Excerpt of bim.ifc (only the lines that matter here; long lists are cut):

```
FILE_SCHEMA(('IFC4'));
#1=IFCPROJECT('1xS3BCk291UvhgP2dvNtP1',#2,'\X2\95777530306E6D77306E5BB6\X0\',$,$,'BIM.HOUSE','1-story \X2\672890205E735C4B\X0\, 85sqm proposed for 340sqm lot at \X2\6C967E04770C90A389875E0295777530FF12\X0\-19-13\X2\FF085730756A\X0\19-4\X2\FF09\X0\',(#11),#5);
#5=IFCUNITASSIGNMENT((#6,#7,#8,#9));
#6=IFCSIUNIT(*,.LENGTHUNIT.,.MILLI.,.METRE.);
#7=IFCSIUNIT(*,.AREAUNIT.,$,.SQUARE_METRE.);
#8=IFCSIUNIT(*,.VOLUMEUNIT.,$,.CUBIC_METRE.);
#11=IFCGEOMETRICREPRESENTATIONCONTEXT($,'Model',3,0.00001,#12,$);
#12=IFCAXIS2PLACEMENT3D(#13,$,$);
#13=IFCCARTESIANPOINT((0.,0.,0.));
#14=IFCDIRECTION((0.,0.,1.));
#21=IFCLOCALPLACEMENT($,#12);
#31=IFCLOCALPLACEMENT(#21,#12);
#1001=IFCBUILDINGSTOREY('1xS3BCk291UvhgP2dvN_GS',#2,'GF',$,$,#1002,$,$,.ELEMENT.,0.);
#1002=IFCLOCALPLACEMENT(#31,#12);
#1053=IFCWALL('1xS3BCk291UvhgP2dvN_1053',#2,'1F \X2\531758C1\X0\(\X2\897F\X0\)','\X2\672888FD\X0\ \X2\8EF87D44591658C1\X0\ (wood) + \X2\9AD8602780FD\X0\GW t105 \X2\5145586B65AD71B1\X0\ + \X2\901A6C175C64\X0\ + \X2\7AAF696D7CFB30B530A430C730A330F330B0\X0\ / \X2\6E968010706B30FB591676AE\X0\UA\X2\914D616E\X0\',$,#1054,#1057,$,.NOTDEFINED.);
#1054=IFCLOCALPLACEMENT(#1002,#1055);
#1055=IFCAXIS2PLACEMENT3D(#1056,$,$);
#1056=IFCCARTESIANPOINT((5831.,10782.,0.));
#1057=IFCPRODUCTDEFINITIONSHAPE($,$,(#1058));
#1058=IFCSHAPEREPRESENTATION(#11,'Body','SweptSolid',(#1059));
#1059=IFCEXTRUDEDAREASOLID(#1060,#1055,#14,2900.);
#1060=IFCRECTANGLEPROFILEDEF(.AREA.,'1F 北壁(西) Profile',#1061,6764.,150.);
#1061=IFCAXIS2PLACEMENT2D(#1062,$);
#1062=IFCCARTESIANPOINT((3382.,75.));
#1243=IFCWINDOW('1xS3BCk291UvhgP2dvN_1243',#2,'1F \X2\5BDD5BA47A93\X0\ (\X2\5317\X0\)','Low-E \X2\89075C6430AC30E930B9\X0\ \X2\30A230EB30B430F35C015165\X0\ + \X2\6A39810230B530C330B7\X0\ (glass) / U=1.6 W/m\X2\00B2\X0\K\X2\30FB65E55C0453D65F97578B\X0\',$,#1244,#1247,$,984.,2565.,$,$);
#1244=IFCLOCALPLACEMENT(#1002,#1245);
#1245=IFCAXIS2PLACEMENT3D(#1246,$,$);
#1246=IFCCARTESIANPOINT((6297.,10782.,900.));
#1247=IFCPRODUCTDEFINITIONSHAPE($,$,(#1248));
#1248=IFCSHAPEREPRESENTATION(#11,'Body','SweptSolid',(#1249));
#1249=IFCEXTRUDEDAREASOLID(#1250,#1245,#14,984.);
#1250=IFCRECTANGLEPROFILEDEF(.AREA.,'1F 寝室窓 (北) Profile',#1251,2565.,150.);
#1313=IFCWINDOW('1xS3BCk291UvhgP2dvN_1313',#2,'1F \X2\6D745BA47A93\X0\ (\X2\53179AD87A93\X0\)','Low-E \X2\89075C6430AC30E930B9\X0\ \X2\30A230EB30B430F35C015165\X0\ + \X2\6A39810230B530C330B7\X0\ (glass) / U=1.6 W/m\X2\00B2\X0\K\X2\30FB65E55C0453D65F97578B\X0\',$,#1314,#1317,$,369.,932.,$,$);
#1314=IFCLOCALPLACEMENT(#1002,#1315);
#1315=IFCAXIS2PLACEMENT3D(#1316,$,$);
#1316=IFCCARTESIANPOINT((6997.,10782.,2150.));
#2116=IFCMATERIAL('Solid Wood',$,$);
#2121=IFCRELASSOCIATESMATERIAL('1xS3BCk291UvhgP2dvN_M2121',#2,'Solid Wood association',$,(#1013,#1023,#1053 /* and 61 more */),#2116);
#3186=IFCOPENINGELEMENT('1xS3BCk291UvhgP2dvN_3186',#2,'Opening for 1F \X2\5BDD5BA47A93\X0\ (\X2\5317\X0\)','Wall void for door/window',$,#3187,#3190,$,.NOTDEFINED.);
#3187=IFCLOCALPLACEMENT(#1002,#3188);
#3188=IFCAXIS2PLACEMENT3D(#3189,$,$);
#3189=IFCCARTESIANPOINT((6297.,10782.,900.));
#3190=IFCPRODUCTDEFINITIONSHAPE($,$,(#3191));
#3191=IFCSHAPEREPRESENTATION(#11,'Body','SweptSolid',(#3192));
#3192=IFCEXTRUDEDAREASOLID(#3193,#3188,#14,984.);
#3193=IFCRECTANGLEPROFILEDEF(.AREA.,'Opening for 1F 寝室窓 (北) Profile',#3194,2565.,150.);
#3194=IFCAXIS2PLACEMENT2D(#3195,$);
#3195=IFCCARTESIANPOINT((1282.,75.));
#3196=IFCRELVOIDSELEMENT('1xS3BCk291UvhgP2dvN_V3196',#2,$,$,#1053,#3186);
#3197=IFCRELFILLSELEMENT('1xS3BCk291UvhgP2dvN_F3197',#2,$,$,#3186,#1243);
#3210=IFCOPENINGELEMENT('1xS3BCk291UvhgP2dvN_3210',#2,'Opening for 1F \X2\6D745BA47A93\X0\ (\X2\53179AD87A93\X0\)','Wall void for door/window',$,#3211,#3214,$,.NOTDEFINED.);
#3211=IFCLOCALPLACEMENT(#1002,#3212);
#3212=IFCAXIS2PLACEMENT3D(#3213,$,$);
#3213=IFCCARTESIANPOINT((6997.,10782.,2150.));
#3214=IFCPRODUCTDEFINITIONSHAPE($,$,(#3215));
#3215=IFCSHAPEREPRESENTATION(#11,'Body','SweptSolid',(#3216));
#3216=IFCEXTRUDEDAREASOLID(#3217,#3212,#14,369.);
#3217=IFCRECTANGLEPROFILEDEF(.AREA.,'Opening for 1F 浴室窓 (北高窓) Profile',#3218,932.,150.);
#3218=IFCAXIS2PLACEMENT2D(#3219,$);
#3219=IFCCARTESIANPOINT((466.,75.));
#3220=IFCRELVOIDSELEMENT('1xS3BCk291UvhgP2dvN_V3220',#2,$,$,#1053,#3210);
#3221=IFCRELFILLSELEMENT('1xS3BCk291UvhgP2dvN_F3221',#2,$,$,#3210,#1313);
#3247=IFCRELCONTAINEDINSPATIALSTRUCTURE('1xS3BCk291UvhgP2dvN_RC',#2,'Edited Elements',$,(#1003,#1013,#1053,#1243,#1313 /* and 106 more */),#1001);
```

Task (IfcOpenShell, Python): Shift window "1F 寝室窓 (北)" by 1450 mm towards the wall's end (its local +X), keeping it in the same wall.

```python
import ifcopenshell
import ifcopenshell.api.geometry
import ifcopenshell.util.placement
import ifcopenshell.util.unit

model = ifcopenshell.open("bim.ifc")
unit_scale = ifcopenshell.util.unit.calculate_unit_scale(model)

window = model.by_guid("1xS3BCk291UvhgP2dvN_1243")
opening = window.FillsVoids[0].RelatingOpeningElement
wall = opening.VoidsElements[0].RelatingBuildingElement

wall_matrix = ifcopenshell.util.placement.get_local_placement(wall.ObjectPlacement)
shift = wall_matrix[:3, 0] * 1.45 / unit_scale
before = ifcopenshell.util.placement.get_local_placement(window.ObjectPlacement)[:3, 3].copy()

# The window is not placed relative to its opening, so move both.
for product in (opening, window):
    matrix = ifcopenshell.util.placement.get_local_placement(product.ObjectPlacement)
    matrix[:3, 3] += shift
    ifcopenshell.api.geometry.edit_object_placement(model, product=product, matrix=matrix, is_si=False)

after = ifcopenshell.util.placement.get_local_placement(window.ObjectPlacement)[:3, 3]
print("window moved by", (after - before).round(3) + 0.0)

model.write("bim_edited.ifc")
```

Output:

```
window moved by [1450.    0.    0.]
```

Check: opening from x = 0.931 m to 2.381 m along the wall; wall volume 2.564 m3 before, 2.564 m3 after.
